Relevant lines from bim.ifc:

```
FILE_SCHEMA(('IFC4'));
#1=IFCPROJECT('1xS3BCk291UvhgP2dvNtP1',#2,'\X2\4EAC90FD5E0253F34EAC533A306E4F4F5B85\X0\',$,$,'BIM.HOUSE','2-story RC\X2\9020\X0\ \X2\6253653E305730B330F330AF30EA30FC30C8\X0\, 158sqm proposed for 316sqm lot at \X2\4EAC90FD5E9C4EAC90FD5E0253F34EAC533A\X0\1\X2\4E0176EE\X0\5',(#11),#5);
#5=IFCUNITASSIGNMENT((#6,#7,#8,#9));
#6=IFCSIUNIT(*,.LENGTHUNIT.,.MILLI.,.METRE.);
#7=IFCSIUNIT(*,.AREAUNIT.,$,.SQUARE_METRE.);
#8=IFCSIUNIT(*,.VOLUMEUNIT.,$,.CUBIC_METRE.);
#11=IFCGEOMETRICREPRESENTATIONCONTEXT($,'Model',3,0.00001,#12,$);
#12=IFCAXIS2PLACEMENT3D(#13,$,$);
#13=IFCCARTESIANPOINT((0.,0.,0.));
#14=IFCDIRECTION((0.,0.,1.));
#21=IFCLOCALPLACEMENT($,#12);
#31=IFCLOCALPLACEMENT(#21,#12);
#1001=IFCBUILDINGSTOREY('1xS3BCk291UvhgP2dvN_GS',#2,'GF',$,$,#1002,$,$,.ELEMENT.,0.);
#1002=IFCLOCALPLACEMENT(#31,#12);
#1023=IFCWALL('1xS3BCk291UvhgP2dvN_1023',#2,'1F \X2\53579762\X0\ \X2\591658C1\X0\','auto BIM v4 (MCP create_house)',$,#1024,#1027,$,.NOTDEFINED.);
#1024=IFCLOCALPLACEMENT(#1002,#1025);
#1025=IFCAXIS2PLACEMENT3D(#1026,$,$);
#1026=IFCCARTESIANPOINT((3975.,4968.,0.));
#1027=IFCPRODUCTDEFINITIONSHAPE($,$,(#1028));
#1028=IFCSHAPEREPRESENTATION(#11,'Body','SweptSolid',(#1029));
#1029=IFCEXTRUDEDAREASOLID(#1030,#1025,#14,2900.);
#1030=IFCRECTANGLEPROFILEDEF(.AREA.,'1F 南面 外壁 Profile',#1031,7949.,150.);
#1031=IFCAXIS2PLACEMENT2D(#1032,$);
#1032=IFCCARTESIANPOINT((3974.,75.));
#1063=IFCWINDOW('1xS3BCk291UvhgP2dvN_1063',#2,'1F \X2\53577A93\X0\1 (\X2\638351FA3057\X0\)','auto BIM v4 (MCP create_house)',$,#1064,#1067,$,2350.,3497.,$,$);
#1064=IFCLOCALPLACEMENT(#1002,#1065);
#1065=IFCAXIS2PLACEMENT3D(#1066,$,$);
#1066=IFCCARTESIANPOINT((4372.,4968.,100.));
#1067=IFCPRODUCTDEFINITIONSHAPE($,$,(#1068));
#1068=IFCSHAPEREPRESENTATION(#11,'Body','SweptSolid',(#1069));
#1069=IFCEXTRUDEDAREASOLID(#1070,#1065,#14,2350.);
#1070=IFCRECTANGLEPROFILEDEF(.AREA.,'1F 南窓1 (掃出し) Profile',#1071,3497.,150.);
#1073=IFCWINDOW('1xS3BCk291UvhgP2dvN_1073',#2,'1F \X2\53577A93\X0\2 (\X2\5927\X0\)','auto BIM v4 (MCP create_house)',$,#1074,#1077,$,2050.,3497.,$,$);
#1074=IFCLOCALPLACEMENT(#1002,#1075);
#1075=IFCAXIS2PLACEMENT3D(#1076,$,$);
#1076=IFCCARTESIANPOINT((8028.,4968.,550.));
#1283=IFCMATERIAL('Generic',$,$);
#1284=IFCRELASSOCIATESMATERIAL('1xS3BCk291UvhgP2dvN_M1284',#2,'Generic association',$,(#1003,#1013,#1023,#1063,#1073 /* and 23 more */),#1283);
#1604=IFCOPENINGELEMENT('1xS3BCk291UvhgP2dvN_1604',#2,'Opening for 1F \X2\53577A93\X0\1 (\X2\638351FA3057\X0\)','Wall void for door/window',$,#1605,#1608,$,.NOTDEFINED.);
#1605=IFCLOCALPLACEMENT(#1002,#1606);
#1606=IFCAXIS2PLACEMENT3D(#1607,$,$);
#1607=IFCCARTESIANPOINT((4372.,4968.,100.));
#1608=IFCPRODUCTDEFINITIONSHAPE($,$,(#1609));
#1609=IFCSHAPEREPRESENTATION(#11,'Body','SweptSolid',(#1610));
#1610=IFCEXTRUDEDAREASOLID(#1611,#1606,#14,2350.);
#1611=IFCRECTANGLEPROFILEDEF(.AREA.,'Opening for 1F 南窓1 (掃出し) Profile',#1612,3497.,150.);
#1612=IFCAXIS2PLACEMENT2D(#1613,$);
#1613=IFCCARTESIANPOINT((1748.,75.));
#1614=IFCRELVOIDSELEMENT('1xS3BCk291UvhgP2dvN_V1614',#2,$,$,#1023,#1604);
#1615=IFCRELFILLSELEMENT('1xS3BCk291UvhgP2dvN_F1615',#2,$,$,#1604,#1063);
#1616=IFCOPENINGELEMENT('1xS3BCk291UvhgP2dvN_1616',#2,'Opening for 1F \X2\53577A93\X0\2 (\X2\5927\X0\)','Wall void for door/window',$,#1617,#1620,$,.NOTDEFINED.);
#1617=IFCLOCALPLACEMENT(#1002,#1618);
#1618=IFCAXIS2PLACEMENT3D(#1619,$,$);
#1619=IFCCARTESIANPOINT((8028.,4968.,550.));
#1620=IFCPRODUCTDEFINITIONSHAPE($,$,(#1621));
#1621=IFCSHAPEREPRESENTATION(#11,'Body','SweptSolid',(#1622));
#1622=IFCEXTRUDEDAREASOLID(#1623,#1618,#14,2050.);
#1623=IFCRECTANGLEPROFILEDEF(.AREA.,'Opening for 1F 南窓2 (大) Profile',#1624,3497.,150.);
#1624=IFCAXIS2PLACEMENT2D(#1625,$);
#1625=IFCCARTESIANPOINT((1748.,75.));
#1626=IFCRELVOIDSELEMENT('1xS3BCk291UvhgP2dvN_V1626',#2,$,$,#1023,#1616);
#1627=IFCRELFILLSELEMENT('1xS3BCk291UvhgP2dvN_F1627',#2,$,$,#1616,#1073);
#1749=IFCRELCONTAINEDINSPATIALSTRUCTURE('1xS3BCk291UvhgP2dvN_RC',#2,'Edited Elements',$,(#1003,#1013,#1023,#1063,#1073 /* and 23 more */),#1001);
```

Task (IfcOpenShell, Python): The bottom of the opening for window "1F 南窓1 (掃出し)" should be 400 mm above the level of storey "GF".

```python
import numpy as np
import ifcopenshell
import ifcopenshell.api.geometry
import ifcopenshell.geom
import ifcopenshell.util.element
import ifcopenshell.util.placement
import ifcopenshell.util.shape
import ifcopenshell.util.unit

model = ifcopenshell.open("bim.ifc")
unit_scale = ifcopenshell.util.unit.calculate_unit_scale(model)

window = model.by_guid("1xS3BCk291UvhgP2dvN_1063")
opening = window.FillsVoids[0].RelatingOpeningElement
storey = ifcopenshell.util.element.get_container(window, ifc_class="IfcBuildingStorey")
level = ifcopenshell.util.placement.get_local_placement(storey.ObjectPlacement)[2, 3]

# The opening's origin need not be at the sill, so measure its lowest point.
shape = ifcopenshell.geom.create_shape(ifcopenshell.geom.settings(), opening)
bottom = ifcopenshell.util.shape.get_shape_bottom_elevation(shape, shape.geometry) / unit_scale
dz = level + 0.4 / unit_scale - bottom

shift = np.array([0.0, 0.0, dz])
# The window is not placed relative to its opening, so move both.
for product in (opening, window):
    matrix = ifcopenshell.util.placement.get_local_placement(product.ObjectPlacement)
    matrix[:3, 3] += shift
    ifcopenshell.api.geometry.edit_object_placement(model, product=product, matrix=matrix, is_si=False)

print(f"moved by {dz * unit_scale:+.3f} m")

model.write("bim_updated.ifc")
```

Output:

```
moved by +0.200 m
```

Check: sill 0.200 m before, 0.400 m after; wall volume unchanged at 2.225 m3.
